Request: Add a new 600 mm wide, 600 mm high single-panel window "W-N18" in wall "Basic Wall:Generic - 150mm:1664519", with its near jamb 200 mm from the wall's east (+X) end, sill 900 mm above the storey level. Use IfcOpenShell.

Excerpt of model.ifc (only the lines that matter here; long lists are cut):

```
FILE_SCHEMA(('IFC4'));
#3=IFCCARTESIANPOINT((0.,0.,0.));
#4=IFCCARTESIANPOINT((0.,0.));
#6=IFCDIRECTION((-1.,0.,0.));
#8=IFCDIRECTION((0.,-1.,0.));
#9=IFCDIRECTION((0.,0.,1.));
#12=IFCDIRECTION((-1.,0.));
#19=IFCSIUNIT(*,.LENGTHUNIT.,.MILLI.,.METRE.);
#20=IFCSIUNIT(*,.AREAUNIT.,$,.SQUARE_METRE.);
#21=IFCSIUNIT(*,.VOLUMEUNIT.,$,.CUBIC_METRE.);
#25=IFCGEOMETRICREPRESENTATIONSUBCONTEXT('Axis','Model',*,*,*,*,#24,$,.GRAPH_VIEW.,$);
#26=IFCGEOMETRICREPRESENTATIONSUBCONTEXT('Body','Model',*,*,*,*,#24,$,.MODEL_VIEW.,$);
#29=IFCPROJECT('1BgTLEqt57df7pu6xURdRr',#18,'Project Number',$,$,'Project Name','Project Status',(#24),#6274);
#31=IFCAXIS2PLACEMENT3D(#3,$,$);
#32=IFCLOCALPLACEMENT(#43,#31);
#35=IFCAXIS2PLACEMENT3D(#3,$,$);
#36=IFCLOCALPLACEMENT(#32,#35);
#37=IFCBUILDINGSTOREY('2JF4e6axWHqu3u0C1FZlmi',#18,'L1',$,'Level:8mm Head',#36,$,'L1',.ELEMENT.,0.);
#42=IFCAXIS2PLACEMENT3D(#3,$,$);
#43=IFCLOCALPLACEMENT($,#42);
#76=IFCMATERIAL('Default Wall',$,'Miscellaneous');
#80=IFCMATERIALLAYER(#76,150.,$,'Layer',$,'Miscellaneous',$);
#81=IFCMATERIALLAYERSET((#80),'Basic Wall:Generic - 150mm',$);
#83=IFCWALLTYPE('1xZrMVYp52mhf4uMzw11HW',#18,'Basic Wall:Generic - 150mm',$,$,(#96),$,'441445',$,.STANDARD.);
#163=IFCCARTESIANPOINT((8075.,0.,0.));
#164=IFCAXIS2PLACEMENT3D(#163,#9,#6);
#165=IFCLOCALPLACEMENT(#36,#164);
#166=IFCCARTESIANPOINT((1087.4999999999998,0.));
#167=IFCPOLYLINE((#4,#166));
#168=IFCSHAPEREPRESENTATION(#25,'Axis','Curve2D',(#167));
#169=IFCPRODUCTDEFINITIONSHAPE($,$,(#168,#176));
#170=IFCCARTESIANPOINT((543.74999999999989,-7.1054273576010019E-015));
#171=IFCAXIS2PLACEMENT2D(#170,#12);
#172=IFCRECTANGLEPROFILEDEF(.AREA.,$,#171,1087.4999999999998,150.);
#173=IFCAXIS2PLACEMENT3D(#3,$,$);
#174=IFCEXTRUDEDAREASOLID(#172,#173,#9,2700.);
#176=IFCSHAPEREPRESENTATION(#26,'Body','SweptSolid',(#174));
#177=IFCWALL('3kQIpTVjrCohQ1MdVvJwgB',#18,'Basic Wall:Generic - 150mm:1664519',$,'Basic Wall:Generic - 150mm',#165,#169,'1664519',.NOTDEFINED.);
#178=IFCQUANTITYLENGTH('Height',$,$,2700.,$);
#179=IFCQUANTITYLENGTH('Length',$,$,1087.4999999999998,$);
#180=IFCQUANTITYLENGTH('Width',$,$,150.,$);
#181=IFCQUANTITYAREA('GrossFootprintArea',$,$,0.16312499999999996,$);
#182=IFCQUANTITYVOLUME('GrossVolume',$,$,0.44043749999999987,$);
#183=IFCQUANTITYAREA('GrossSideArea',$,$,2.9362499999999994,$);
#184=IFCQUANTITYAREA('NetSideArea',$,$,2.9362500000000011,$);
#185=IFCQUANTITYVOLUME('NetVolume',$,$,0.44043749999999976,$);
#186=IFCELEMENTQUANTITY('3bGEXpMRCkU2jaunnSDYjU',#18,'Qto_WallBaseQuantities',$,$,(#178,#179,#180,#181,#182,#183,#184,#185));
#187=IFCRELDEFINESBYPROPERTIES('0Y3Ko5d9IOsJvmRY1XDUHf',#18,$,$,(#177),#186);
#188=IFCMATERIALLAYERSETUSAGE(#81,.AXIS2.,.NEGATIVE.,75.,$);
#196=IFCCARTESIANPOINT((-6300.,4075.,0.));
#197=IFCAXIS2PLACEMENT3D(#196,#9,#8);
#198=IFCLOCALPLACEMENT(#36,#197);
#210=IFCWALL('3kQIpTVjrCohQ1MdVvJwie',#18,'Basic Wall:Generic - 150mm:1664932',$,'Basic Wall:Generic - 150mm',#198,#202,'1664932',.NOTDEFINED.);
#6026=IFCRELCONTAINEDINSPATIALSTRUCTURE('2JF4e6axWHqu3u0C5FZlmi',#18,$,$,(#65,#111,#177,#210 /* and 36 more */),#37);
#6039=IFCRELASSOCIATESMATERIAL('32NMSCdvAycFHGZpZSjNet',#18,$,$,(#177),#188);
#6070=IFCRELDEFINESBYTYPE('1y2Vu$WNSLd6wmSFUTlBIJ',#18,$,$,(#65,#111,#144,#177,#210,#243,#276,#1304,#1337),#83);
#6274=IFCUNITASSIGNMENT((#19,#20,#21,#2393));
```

```python
import numpy as np
import ifcopenshell
import ifcopenshell.api.feature
import ifcopenshell.api.geometry
import ifcopenshell.api.pset
import ifcopenshell.api.root
import ifcopenshell.api.spatial
import ifcopenshell.geom
import ifcopenshell.util.element
import ifcopenshell.util.placement
import ifcopenshell.util.representation
import ifcopenshell.util.shape
import ifcopenshell.util.unit

model = ifcopenshell.open("model.ifc")
unit_scale = ifcopenshell.util.unit.calculate_unit_scale(model)
area_scale = ifcopenshell.util.unit.calculate_unit_scale(model, "AREAUNIT")
volume_scale = ifcopenshell.util.unit.calculate_unit_scale(model, "VOLUMEUNIT")
settings = ifcopenshell.geom.settings()


def volume(element):
    """Net volume in cubic metres, openings subtracted."""
    shape = ifcopenshell.geom.create_shape(settings, element)
    return ifcopenshell.util.shape.get_volume(shape.geometry)


wall = model.by_guid("3kQIpTVjrCohQ1MdVvJwgB")
storey = ifcopenshell.util.element.get_container(wall, ifc_class="IfcBuildingStorey")
context = ifcopenshell.util.representation.get_context(model, "Model", "Body", "MODEL_VIEW")
before = volume(wall)

width, height, from_end, sill = 0.6, 0.6, 0.2, 0.9  # metres

# The wall runs along its own X axis, and the end named is its -X end.
wall_shape = ifcopenshell.geom.create_shape(settings, wall)
x, y, z = ifcopenshell.util.shape.get_vertices(wall_shape.geometry).T
start = x.min() + from_end
face, thickness = float(y.min()), float(y.max() - y.min())
wall_matrix = ifcopenshell.util.placement.get_local_placement(wall.ObjectPlacement)
level = ifcopenshell.util.placement.get_local_placement(storey.ObjectPlacement)[2, 3]


def in_wall(x, y):
    """Placement at x, y metres in the wall's axes, at sill height."""
    matrix = wall_matrix.copy()
    matrix[:, 3] = wall_matrix @ np.array([x / unit_scale, y / unit_scale, 0.0, 1.0])
    matrix[2, 3] = level + sill / unit_scale
    return matrix


# Opening: a box that overshoots both wall faces by 50 mm.
opening = ifcopenshell.api.root.create_entity(model, ifc_class="IfcOpeningElement", predefined_type="OPENING")
box = ifcopenshell.api.geometry.add_wall_representation(
    model, context=context, length=width, height=height, thickness=thickness + 0.1
)
ifcopenshell.api.geometry.assign_representation(model, product=opening, representation=box)
ifcopenshell.api.geometry.edit_object_placement(model, product=opening, matrix=in_wall(start, face - 0.05), is_si=False)
ifcopenshell.api.feature.add_feature(model, feature=opening, element=wall)

window = ifcopenshell.api.root.create_entity(model, ifc_class="IfcWindow", name="W-N18", predefined_type="WINDOW")
window.OverallWidth, window.OverallHeight = width / unit_scale, height / unit_scale
window.PartitioningType = "SINGLE_PANEL"
body = ifcopenshell.api.geometry.add_window_representation(
    model,
    context=context,
    overall_width=window.OverallWidth,
    overall_height=window.OverallHeight,
    partition_type="SINGLE_PANEL",
)
ifcopenshell.api.geometry.assign_representation(model, product=window, representation=body)
ifcopenshell.api.spatial.assign_container(model, products=[window], relating_structure=storey)
ifcopenshell.api.feature.add_filling(model, opening=opening, element=window)

# Centre the window in the wall's thickness.
ifcopenshell.api.geometry.edit_object_placement(model, product=window, matrix=in_wall(start, face), is_si=False)
window_shape = ifcopenshell.geom.create_shape(settings, window)
depth = ifcopenshell.util.shape.get_vertices(window_shape.geometry)[:, 1]
offset = face + thickness / 2 - (depth.min() + depth.max()) / 2
ifcopenshell.api.geometry.edit_object_placement(model, product=window, matrix=in_wall(start, offset), is_si=False)

after = volume(wall)

# Update the wall's stored quantities.
qto = model.by_id(ifcopenshell.util.element.get_pset(wall, "Qto_WallBaseQuantities", should_inherit=False)["id"])
ifcopenshell.api.pset.edit_qto(model, qto=qto, properties={
    "NetSideArea": after / thickness / area_scale,
    "NetVolume": after / volume_scale,
})

print(f"wall volume {before:.3f} -> {after:.3f} m3")

model.write("model_edited.ifc")
```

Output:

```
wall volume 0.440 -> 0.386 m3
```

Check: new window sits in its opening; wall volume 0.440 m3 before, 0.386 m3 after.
